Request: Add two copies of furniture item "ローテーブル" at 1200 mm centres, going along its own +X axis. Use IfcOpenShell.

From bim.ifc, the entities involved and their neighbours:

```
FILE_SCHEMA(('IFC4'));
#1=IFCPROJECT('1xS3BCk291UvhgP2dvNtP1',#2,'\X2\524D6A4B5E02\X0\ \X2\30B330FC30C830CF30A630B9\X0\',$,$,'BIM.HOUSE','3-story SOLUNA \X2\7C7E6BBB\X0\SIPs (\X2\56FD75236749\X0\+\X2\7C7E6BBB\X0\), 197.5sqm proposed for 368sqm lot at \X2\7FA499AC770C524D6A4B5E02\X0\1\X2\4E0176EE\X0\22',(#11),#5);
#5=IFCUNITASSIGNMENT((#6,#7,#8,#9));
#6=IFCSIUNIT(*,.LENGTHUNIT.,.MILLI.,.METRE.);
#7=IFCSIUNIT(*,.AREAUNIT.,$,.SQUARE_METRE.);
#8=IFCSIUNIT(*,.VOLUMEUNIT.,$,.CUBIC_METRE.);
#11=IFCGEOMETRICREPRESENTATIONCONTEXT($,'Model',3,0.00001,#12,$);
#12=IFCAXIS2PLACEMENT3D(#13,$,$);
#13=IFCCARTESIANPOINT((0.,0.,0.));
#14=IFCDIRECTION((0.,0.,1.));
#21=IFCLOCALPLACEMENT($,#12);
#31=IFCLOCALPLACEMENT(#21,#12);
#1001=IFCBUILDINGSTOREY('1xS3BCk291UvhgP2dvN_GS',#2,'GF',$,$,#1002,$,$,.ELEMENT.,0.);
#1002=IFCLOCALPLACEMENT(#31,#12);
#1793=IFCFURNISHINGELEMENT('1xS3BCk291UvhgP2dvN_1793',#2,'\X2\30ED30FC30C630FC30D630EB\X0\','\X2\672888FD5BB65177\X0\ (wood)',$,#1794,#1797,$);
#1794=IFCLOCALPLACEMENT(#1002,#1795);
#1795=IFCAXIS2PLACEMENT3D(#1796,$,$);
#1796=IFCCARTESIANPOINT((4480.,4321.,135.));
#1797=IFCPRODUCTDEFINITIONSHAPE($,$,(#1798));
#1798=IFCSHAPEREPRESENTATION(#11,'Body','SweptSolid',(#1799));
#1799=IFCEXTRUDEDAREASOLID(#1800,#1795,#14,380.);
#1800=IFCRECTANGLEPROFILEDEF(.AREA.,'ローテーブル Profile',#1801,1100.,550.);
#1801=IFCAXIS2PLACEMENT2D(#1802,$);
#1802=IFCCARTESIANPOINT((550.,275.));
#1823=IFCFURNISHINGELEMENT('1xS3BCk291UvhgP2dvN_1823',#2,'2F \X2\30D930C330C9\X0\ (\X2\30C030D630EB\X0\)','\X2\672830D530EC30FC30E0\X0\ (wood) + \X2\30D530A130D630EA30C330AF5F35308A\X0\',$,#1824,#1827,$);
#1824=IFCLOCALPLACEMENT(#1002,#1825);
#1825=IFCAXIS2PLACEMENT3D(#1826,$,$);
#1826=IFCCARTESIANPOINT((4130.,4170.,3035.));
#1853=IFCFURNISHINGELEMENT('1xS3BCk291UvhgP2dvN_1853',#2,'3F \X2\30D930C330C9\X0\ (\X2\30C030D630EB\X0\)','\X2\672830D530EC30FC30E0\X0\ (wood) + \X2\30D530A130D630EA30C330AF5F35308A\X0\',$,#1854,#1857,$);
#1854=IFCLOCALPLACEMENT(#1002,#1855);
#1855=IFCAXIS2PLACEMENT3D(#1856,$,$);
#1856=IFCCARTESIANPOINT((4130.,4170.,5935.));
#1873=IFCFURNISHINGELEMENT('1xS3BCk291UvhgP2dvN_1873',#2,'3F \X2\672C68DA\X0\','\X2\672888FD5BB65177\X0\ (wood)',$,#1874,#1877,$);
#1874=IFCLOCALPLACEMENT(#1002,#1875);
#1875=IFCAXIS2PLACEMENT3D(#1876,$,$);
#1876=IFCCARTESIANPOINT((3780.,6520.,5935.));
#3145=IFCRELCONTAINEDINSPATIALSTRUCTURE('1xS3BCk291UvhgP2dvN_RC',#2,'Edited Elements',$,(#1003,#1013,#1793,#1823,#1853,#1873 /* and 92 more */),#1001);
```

```python
import ifcopenshell
import ifcopenshell.api.geometry
import ifcopenshell.api.root
import ifcopenshell.util.element
import ifcopenshell.util.placement
import ifcopenshell.util.unit

model = ifcopenshell.open("bim.ifc")
unit_scale = ifcopenshell.util.unit.calculate_unit_scale(model)


def reuse_history(source, copy):
    """copy_class also copies each property set's owner history, people and application; keep the originals."""
    for rel in copy.IsDefinedBy:
        if rel.is_a("IfcRelDefinesByProperties") and (history := rel.RelatingPropertyDefinition.OwnerHistory):
            rel.RelatingPropertyDefinition.OwnerHistory = source.OwnerHistory
            ifcopenshell.util.element.remove_deep2(model, history)


source = model.by_guid("1xS3BCk291UvhgP2dvN_1793")
base = ifcopenshell.util.placement.get_local_placement(source.ObjectPlacement)
step = base[:3, 0] * 1.2 / unit_scale

for i in range(1, 3):
    copy = ifcopenshell.api.root.copy_class(model, product=source)
    copy.Representation = ifcopenshell.util.element.copy_deep(
        model, source.Representation, exclude=["IfcGeometricRepresentationContext", "IfcRepresentationMap"]
    )
    reuse_history(source, copy)
    matrix = base.copy()
    matrix[:3, 3] += i * step
    print("added at", matrix[:3, 3].round(3) + 0.0)
    ifcopenshell.api.geometry.edit_object_placement(model, product=copy, matrix=matrix, is_si=False)

model.write("bim_v2.ifc")
```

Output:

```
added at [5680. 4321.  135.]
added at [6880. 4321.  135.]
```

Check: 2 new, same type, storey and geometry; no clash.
